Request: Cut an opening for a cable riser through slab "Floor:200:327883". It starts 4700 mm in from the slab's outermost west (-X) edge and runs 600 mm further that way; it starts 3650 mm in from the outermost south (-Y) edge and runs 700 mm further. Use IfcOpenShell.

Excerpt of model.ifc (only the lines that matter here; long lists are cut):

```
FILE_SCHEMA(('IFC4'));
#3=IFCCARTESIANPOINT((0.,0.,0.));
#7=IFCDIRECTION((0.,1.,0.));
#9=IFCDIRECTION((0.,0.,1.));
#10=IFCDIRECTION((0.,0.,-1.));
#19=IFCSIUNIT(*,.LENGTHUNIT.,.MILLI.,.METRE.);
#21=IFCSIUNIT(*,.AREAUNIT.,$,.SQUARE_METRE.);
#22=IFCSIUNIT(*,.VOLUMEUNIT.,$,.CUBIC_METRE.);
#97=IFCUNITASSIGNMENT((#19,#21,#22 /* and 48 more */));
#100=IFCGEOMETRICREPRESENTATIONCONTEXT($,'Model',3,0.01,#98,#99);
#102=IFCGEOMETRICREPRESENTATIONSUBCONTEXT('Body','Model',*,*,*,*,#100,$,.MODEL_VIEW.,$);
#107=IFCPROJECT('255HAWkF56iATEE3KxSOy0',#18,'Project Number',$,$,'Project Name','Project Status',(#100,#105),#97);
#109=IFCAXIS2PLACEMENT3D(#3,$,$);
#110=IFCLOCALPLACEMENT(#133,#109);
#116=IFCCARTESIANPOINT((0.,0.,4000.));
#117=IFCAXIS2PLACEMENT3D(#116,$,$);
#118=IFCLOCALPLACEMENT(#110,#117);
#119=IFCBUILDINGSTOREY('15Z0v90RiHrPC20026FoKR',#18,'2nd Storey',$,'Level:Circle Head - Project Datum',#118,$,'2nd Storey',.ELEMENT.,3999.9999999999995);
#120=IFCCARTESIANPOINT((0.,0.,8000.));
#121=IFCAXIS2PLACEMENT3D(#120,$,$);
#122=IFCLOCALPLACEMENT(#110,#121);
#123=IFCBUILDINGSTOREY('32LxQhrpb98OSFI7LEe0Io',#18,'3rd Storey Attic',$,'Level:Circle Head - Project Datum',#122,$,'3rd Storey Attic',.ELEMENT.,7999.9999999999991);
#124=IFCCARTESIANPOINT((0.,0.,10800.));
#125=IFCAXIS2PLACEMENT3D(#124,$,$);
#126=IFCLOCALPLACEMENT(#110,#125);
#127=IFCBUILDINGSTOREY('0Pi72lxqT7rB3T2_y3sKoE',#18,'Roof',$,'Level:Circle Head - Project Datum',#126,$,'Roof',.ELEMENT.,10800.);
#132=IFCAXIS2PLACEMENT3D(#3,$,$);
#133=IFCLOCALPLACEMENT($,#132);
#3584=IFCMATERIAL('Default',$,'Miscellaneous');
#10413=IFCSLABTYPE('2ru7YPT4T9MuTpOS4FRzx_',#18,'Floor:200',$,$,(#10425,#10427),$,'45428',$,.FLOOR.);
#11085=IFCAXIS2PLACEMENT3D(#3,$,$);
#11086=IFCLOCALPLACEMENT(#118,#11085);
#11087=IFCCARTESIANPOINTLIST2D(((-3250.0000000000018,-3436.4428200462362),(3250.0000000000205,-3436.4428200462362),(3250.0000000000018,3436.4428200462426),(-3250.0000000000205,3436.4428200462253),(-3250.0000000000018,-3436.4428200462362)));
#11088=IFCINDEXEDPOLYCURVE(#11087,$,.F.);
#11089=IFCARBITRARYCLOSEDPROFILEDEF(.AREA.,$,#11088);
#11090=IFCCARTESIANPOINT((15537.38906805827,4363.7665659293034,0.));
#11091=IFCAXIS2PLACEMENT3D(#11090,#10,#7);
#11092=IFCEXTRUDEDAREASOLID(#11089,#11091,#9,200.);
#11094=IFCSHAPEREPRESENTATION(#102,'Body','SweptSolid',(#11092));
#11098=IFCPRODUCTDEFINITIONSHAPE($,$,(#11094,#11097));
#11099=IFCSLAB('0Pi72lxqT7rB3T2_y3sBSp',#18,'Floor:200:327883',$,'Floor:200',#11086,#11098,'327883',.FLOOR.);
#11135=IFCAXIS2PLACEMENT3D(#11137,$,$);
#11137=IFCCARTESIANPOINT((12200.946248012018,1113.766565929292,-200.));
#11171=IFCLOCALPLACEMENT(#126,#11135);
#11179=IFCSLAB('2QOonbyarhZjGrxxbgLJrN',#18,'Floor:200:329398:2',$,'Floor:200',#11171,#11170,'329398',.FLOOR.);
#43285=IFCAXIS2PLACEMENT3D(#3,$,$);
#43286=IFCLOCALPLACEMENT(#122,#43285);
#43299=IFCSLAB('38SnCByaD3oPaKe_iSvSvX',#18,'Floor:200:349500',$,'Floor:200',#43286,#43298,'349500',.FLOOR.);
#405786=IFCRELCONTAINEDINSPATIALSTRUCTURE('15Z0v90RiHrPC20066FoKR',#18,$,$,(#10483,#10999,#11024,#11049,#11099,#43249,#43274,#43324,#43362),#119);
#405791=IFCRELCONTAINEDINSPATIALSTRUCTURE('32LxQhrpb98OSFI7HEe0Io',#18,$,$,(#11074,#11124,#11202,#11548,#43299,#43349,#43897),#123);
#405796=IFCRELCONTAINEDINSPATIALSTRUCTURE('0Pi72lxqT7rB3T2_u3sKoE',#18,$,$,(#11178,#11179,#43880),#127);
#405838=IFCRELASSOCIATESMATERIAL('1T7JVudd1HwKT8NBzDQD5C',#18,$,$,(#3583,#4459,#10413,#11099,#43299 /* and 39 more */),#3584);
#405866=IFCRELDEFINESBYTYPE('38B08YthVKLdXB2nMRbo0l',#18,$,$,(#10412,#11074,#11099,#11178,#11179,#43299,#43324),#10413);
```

```python
import numpy as np
import ifcopenshell
import ifcopenshell.api.feature
import ifcopenshell.api.geometry
import ifcopenshell.api.root
import ifcopenshell.geom
import ifcopenshell.util.placement
import ifcopenshell.util.representation
import ifcopenshell.util.shape
import ifcopenshell.util.unit

model = ifcopenshell.open("model.ifc")
unit_scale = ifcopenshell.util.unit.calculate_unit_scale(model)
settings = ifcopenshell.geom.settings()


def volume(element):
    """Net volume in cubic metres, openings subtracted."""
    shape = ifcopenshell.geom.create_shape(settings, element)
    return ifcopenshell.util.shape.get_volume(shape.geometry)


slab = model.by_guid("0Pi72lxqT7rB3T2_y3sBSp")
before = volume(slab)

# Extent in the slab's own axes, in metres. The edges named are its -X and -Y sides.
slab_shape = ifcopenshell.geom.create_shape(settings, slab)
vertices = ifcopenshell.util.shape.get_vertices(slab_shape.geometry)
x_min, y_min, bottom = vertices.min(axis=0)
top = vertices[:, 2].max()

opening = ifcopenshell.api.root.create_entity(model, ifc_class="IfcOpeningElement", name="Cable riser opening", predefined_type="OPENING")
context = ifcopenshell.util.representation.get_context(model, "Model", "Body", "MODEL_VIEW")
width, depth = 0.6, 0.7
outline = [(0.0, 0.0), (width, 0.0), (width, depth), (0.0, depth), (0.0, 0.0)]
# Overshoot both faces by 50 mm so the cut is clean.
shape = ifcopenshell.api.geometry.add_slab_representation(
    model, context=context, depth=top - bottom + 0.1, polyline=outline
)
ifcopenshell.api.geometry.assign_representation(model, product=opening, representation=shape)

matrix = ifcopenshell.util.placement.get_local_placement(slab.ObjectPlacement)
matrix[:, 3] = matrix @ np.append(np.array([x_min + 4.7, y_min + 3.65, bottom - 0.05]) / unit_scale, 1.0)
ifcopenshell.api.geometry.edit_object_placement(model, product=opening, matrix=matrix, is_si=False)
ifcopenshell.api.feature.add_feature(model, feature=opening, element=slab)

after = volume(slab)

print(f"slab volume {before:.3f} -> {after:.3f} m3")

model.write("model_v2.ifc")
```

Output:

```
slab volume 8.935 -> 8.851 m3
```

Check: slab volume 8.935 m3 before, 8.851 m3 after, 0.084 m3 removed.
